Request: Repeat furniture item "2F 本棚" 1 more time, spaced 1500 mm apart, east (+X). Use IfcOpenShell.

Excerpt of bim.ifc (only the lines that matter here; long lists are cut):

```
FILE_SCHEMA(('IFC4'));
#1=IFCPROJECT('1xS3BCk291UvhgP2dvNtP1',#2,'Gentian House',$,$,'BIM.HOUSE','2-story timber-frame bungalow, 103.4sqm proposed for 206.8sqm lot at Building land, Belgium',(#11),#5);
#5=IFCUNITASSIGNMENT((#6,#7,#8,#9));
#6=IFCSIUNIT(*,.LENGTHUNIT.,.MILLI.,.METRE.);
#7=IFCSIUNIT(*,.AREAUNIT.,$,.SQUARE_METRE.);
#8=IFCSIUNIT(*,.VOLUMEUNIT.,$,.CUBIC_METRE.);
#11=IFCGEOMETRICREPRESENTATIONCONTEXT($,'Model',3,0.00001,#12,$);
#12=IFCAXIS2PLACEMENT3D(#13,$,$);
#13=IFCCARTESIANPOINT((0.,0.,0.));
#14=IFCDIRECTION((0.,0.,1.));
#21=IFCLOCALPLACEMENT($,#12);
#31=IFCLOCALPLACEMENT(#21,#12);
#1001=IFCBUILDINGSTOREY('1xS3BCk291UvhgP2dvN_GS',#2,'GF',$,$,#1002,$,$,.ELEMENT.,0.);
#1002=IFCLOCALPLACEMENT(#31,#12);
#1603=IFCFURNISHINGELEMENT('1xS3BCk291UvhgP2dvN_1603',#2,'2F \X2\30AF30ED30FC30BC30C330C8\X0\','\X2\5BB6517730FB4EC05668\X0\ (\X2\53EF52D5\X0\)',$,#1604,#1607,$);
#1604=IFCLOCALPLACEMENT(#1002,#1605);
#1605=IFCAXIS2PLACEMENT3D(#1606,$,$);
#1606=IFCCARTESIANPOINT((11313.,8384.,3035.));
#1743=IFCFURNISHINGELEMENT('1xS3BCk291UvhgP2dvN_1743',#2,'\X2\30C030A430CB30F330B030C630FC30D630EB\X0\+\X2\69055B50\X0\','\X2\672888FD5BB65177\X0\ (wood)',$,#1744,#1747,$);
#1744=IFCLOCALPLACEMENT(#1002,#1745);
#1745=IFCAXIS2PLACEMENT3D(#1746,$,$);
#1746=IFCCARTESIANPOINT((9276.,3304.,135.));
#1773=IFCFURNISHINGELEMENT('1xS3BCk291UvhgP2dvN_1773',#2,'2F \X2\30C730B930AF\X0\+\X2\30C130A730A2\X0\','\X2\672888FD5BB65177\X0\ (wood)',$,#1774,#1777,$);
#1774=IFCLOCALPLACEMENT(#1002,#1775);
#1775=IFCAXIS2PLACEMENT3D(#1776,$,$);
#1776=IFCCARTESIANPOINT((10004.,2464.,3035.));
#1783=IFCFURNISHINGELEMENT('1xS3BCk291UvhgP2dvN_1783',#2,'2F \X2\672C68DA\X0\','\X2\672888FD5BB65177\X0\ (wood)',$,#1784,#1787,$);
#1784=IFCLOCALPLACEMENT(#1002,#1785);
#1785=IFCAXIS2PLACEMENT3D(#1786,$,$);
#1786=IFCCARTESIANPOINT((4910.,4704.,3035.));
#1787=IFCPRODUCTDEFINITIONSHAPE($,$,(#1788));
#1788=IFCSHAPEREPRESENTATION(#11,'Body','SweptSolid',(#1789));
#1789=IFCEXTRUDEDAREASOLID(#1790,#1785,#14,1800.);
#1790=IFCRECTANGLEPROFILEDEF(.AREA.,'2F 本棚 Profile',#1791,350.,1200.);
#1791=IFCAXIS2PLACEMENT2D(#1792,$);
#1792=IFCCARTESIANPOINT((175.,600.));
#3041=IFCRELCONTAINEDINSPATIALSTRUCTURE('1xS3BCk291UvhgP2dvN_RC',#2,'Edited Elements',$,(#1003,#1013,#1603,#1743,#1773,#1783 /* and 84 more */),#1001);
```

```python
import numpy as np
import ifcopenshell
import ifcopenshell.api.geometry
import ifcopenshell.api.root
import ifcopenshell.util.element
import ifcopenshell.util.placement

model = ifcopenshell.open("bim.ifc")


def reuse_history(source, copy):
    """copy_class also copies each property set's owner history, people and application; keep the originals."""
    for rel in copy.IsDefinedBy:
        if rel.is_a("IfcRelDefinesByProperties") and (history := rel.RelatingPropertyDefinition.OwnerHistory):
            rel.RelatingPropertyDefinition.OwnerHistory = source.OwnerHistory
            ifcopenshell.util.element.remove_deep2(model, history)


source = model.by_guid("1xS3BCk291UvhgP2dvN_1783")
base = ifcopenshell.util.placement.get_local_placement(source.ObjectPlacement)
step = np.array([1.0, 0.0, 0.0]) * 1500.0

for i in range(1, 2):
    copy = ifcopenshell.api.root.copy_class(model, product=source)
    copy.Representation = ifcopenshell.util.element.copy_deep(
        model, source.Representation, exclude=["IfcGeometricRepresentationContext", "IfcRepresentationMap"]
    )
    reuse_history(source, copy)
    matrix = base.copy()
    matrix[:3, 3] += i * step
    print("added at", matrix[:3, 3].round(3) + 0.0)
    ifcopenshell.api.geometry.edit_object_placement(model, product=copy, matrix=matrix, is_si=False)

model.write("bim_updated.ifc")
```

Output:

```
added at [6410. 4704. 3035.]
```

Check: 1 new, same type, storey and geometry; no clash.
